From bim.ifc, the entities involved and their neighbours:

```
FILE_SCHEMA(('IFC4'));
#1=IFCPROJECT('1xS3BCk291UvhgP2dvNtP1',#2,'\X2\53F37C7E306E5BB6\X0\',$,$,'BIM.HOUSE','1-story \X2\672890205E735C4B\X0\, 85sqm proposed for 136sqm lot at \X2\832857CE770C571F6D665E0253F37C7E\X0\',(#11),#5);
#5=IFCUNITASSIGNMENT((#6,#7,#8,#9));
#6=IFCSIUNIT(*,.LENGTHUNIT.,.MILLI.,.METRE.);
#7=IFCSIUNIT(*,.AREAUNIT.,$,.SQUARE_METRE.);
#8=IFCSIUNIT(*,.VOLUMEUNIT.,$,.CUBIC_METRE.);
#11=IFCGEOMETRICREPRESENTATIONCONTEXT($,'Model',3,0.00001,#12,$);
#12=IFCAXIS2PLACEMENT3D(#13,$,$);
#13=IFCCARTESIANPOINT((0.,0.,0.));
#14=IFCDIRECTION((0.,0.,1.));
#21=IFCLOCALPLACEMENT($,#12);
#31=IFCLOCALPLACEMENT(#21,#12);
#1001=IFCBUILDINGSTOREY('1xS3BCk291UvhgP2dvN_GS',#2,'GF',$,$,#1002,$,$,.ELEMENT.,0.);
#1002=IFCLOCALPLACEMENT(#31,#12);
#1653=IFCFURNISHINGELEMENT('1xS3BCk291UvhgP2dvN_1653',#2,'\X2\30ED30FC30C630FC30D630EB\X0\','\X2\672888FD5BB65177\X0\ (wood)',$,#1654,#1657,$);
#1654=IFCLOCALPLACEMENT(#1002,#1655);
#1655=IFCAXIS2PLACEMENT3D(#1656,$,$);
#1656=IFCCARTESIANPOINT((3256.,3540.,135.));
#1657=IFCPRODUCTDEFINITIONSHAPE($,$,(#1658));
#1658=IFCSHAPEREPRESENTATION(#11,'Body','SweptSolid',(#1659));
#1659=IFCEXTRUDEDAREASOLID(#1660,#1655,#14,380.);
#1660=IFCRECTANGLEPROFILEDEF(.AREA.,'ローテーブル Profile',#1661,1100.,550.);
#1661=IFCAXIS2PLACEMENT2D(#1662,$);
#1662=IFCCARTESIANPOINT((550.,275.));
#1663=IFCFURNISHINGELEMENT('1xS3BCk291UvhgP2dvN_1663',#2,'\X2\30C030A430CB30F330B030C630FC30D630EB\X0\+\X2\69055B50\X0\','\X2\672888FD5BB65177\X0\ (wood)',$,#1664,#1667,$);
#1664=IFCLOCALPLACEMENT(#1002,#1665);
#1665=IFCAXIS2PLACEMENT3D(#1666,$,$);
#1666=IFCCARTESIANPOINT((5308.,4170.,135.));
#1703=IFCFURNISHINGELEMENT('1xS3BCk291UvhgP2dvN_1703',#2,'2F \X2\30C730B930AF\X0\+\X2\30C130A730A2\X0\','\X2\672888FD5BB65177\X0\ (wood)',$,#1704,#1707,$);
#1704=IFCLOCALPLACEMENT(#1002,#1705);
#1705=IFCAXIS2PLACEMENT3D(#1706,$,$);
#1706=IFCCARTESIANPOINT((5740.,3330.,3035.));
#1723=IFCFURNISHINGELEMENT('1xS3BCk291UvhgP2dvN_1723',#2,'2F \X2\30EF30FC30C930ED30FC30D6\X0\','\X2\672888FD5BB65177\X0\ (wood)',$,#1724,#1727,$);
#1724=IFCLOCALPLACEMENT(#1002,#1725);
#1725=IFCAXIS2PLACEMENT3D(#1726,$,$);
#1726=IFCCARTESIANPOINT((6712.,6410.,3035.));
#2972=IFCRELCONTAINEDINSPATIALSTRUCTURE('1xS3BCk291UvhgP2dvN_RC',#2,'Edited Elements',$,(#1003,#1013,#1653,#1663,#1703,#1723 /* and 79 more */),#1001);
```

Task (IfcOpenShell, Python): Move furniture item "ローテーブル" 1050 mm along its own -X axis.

```python
import ifcopenshell
import ifcopenshell.api.geometry
import ifcopenshell.util.placement
import ifcopenshell.util.unit

model = ifcopenshell.open("bim.ifc")
unit_scale = ifcopenshell.util.unit.calculate_unit_scale(model)

item = model.by_guid("1xS3BCk291UvhgP2dvN_1653")
matrix = ifcopenshell.util.placement.get_local_placement(item.ObjectPlacement)
matrix[:3, 3] -= matrix[:3, 0] * 1.05 / unit_scale
ifcopenshell.api.geometry.edit_object_placement(model, product=item, matrix=matrix, is_si=False)

print(ifcopenshell.util.placement.get_local_placement(item.ObjectPlacement).round(3) + 0.0)

model.write("bim_rev.ifc")
```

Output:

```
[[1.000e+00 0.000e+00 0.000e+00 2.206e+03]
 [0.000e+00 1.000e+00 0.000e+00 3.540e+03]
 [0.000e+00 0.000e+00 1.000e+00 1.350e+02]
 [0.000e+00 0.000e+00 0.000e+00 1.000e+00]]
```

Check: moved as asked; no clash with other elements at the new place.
